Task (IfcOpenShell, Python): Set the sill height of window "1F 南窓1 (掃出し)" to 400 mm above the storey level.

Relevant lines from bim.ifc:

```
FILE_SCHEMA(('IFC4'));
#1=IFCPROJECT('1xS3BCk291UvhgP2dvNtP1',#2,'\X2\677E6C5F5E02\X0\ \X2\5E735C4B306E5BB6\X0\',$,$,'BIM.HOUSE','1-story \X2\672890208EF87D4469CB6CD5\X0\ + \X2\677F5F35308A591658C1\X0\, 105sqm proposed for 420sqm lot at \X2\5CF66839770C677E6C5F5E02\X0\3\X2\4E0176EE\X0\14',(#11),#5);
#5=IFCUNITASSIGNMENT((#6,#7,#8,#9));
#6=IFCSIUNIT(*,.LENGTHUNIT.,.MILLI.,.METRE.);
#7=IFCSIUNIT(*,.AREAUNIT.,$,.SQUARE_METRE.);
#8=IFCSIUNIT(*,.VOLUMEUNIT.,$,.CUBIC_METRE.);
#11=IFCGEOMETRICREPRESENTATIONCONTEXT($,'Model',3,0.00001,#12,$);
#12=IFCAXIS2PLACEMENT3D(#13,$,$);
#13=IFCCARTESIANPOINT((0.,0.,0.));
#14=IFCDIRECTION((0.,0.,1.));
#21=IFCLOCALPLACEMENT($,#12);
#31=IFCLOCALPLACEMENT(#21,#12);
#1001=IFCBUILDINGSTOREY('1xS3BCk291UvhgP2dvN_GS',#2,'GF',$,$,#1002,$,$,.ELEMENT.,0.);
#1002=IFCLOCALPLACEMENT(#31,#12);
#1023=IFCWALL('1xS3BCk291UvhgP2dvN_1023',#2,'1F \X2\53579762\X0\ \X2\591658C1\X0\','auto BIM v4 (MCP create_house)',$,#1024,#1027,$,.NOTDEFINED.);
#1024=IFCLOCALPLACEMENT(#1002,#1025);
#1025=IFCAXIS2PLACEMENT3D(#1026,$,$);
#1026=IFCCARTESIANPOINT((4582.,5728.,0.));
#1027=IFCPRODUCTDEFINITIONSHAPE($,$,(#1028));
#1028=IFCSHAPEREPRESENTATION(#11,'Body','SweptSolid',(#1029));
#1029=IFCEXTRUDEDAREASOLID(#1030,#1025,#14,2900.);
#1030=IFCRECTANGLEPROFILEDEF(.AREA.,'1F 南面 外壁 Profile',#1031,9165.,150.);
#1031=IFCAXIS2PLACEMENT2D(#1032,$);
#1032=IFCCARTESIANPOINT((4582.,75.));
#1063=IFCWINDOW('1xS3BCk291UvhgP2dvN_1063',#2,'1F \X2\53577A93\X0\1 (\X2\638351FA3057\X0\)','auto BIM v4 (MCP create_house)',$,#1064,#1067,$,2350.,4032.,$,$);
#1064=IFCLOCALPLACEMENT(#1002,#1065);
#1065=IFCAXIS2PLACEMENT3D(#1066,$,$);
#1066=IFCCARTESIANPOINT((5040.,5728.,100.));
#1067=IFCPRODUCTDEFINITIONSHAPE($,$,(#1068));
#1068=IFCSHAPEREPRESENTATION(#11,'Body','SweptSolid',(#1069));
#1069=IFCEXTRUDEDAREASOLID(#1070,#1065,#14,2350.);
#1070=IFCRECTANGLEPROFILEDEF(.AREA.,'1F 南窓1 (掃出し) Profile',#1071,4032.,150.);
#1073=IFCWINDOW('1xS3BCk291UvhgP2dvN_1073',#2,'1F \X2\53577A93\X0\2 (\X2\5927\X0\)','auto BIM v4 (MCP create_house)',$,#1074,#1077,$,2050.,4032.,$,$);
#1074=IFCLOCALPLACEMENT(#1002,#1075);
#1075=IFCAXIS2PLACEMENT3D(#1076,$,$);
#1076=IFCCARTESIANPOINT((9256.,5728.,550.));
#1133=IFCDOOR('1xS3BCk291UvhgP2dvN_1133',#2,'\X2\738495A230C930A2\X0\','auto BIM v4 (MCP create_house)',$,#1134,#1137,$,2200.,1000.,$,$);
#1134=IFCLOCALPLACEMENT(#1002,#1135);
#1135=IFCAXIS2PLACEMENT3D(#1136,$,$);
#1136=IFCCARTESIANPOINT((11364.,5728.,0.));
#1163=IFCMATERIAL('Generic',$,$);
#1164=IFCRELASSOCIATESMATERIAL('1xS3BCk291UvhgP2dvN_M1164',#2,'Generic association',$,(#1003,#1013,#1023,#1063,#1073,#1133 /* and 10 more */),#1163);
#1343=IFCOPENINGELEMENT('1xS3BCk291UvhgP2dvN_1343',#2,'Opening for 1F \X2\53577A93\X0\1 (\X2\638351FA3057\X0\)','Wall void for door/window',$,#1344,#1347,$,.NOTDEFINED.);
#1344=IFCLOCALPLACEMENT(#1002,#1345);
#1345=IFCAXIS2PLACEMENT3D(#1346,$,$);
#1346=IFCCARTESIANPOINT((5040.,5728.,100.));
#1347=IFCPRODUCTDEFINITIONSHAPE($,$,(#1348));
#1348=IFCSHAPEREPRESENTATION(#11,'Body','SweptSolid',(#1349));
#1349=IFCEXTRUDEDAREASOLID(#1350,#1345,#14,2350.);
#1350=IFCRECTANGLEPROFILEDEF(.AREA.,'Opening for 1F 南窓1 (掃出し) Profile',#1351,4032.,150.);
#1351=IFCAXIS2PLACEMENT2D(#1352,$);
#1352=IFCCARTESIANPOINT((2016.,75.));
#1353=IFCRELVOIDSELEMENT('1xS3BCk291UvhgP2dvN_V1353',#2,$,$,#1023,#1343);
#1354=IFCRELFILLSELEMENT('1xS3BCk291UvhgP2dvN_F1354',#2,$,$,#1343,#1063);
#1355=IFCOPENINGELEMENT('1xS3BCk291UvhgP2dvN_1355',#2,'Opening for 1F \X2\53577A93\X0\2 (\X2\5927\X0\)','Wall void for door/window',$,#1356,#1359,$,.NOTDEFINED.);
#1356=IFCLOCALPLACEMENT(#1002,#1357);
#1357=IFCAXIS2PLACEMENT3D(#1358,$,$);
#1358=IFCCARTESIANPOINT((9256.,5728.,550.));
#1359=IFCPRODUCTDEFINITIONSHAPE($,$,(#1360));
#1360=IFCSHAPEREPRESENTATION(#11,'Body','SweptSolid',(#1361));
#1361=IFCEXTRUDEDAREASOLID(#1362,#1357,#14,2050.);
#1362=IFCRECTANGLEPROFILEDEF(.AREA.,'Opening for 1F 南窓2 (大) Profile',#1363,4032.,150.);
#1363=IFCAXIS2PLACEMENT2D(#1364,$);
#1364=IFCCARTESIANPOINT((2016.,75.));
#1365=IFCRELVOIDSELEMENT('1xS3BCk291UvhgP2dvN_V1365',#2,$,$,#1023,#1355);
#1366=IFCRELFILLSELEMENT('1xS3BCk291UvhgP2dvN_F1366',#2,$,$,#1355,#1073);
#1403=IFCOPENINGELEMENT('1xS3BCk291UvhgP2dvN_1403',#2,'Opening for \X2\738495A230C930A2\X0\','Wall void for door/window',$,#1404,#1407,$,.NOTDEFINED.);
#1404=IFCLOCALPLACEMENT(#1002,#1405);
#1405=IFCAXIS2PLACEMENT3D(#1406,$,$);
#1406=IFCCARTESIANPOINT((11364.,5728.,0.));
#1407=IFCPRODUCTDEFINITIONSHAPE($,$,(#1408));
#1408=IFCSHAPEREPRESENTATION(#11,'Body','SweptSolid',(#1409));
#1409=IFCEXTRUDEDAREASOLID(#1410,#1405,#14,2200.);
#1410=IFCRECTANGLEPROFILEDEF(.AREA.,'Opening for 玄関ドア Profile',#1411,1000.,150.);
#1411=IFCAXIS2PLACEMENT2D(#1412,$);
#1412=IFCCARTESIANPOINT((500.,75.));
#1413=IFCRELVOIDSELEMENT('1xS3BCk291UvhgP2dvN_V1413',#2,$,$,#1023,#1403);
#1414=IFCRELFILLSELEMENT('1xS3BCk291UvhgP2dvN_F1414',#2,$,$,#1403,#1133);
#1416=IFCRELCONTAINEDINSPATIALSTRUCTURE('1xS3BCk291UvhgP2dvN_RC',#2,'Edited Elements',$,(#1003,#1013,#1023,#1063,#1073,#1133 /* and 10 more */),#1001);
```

```python
import numpy as np
import ifcopenshell
import ifcopenshell.api.geometry
import ifcopenshell.geom
import ifcopenshell.util.element
import ifcopenshell.util.placement
import ifcopenshell.util.shape
import ifcopenshell.util.unit

model = ifcopenshell.open("bim.ifc")
unit_scale = ifcopenshell.util.unit.calculate_unit_scale(model)

window = model.by_id(1063)
opening = window.FillsVoids[0].RelatingOpeningElement
storey = ifcopenshell.util.element.get_container(window, ifc_class="IfcBuildingStorey")
level = ifcopenshell.util.placement.get_local_placement(storey.ObjectPlacement)[2, 3]

# The opening's origin need not be at the sill, so measure its lowest point.
shape = ifcopenshell.geom.create_shape(ifcopenshell.geom.settings(), opening)
bottom = ifcopenshell.util.shape.get_shape_bottom_elevation(shape, shape.geometry) / unit_scale
dz = level + 0.4 / unit_scale - bottom

shift = np.array([0.0, 0.0, dz])
# The window is not placed relative to its opening, so move both.
for product in (opening, window):
    matrix = ifcopenshell.util.placement.get_local_placement(product.ObjectPlacement)
    matrix[:3, 3] += shift
    ifcopenshell.api.geometry.edit_object_placement(model, product=product, matrix=matrix, is_si=False)

print(f"moved by {dz * unit_scale:+.3f} m")

model.write("bim_edited.ifc")
```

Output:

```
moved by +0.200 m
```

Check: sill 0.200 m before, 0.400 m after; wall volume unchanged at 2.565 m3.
